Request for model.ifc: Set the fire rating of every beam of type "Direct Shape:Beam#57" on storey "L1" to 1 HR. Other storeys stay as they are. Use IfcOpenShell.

First a look at what the model holds.

```python
import ifcopenshell
import ifcopenshell.util.element

model = ifcopenshell.open("model.ifc")
print(model.schema)
storey = next(s for s in model.by_type("IfcBuildingStorey") if s.Name == "L1")
beams = [e for e in ifcopenshell.util.element.get_decomposition(storey) if e.is_a("IfcBeam")]
seen = {}
for e in beams:
    element_type = ifcopenshell.util.element.get_type(e)
    key = (element_type.Name if element_type != e and element_type else None, ifcopenshell.util.element.get_pset(e, "Pset_BeamCommon", "FireRating"))
    seen[key] = seen.get(key, 0) + 1
for (name, value), count in sorted(seen.items(), key=str):
    print(count, "x", name, "|", value)
```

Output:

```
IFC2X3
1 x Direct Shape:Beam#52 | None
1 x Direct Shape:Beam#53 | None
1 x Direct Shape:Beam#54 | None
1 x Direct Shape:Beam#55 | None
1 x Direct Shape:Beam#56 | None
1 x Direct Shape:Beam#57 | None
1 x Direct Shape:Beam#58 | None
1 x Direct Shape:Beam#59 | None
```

```python
import ifcopenshell
import ifcopenshell.api.pset
import ifcopenshell.util.element

model = ifcopenshell.open("model.ifc")

storey = next(s for s in model.by_type("IfcBuildingStorey") if s.Name == "L1")
beams = [e for e in ifcopenshell.util.element.get_decomposition(storey) if e.is_a("IfcBeam")]

count = 0
for e in beams:
    element_type = ifcopenshell.util.element.get_type(e)
    if element_type in (None, e) or element_type.Name != "Direct Shape:Beam#57":
        continue
    # add_pset returns the element's existing set when there is one.
    pset = ifcopenshell.api.pset.add_pset(model, product=e, name="Pset_BeamCommon")
    ifcopenshell.api.pset.edit_pset(model, pset=pset, properties={"FireRating": "1 HR"})
    count += 1

print(count, "beams updated")

model.write("model_edited.ifc")
```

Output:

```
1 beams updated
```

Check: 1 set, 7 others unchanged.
